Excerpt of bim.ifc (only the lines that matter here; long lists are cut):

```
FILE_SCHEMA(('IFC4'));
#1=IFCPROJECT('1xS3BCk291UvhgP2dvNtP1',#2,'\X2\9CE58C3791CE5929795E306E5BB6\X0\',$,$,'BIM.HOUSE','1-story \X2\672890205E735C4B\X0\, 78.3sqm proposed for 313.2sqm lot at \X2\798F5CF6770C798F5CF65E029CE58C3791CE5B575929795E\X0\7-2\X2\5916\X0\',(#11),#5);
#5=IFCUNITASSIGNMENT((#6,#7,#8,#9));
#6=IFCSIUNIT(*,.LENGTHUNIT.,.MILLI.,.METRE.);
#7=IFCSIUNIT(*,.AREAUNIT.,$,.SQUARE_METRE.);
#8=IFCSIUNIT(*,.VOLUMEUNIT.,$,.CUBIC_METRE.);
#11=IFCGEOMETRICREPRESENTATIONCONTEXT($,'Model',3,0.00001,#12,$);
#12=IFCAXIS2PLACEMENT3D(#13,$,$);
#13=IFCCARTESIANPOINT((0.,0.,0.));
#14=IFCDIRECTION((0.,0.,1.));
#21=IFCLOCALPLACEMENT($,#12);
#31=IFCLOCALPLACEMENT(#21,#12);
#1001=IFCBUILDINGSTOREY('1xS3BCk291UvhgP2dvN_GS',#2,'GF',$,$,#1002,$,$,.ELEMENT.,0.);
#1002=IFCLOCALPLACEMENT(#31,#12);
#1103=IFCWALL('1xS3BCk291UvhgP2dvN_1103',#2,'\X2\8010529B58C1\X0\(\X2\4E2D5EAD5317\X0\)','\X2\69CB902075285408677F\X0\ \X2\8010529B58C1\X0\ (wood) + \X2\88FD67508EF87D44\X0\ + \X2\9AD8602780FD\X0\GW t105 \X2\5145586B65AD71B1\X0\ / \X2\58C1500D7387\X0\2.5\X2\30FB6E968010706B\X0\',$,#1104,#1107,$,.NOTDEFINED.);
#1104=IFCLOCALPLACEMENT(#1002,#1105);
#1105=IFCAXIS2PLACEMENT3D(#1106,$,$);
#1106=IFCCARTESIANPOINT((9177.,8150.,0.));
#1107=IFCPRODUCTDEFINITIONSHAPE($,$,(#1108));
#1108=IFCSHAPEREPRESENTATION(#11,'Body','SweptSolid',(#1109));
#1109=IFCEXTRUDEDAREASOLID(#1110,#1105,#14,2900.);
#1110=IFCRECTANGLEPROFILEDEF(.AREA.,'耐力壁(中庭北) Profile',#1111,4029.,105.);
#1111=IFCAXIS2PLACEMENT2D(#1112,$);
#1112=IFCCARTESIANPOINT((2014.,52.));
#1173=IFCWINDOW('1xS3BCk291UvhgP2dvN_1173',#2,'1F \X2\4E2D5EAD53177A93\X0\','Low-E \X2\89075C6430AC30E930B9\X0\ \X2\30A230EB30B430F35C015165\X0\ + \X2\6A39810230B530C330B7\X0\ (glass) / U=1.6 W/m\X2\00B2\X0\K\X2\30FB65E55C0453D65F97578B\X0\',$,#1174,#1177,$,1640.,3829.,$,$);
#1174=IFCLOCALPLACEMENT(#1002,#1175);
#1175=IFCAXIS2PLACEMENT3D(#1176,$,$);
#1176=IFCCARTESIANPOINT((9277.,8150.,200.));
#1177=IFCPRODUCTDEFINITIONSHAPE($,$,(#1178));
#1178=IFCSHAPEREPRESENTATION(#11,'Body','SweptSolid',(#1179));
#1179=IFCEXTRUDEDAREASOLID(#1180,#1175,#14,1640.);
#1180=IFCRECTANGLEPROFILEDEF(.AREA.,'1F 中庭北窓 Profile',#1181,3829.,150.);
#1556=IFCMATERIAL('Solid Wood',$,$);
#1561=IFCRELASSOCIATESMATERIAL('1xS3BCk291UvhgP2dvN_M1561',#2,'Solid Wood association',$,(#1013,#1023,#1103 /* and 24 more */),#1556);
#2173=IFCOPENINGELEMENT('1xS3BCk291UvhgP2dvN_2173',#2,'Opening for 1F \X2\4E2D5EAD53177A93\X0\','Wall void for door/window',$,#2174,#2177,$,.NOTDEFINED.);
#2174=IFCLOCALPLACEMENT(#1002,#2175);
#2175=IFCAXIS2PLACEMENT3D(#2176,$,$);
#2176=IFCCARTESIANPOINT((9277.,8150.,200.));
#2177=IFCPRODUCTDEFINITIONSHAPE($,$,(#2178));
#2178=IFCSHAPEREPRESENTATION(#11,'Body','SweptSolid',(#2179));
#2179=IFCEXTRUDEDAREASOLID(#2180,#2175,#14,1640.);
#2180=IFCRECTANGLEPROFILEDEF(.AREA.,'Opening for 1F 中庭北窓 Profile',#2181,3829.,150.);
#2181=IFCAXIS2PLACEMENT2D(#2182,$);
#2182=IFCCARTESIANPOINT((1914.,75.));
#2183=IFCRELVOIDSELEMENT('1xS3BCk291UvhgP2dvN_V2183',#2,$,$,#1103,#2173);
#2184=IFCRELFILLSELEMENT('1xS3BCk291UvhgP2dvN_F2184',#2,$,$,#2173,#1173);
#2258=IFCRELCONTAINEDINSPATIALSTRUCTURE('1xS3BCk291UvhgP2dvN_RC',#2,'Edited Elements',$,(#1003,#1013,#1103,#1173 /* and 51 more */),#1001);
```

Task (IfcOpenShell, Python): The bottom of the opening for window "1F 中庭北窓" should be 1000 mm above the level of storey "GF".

```python
import numpy as np
import ifcopenshell
import ifcopenshell.api.geometry
import ifcopenshell.geom
import ifcopenshell.util.element
import ifcopenshell.util.placement
import ifcopenshell.util.shape
import ifcopenshell.util.unit

model = ifcopenshell.open("bim.ifc")
unit_scale = ifcopenshell.util.unit.calculate_unit_scale(model)

window = model.by_guid("1xS3BCk291UvhgP2dvN_1173")
opening = window.FillsVoids[0].RelatingOpeningElement
storey = ifcopenshell.util.element.get_container(window, ifc_class="IfcBuildingStorey")
level = ifcopenshell.util.placement.get_local_placement(storey.ObjectPlacement)[2, 3]

# The opening's origin need not be at the sill, so measure its lowest point.
shape = ifcopenshell.geom.create_shape(ifcopenshell.geom.settings(), opening)
bottom = ifcopenshell.util.shape.get_shape_bottom_elevation(shape, shape.geometry) / unit_scale
dz = level + 1 / unit_scale - bottom

shift = np.array([0.0, 0.0, dz])
# The window is not placed relative to its opening, so move both.
for product in (opening, window):
    matrix = ifcopenshell.util.placement.get_local_placement(product.ObjectPlacement)
    matrix[:3, 3] += shift
    ifcopenshell.api.geometry.edit_object_placement(model, product=product, matrix=matrix, is_si=False)

print(f"moved by {dz * unit_scale:+.3f} m")

model.write("bim_v2.ifc")
```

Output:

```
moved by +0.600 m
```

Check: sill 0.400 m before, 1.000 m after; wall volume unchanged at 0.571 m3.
